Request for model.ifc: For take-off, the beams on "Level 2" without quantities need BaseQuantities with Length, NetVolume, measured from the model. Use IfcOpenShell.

First a look at what the model holds.

```python
import ifcopenshell
import ifcopenshell.util.element
import ifcopenshell.util.unit

model = ifcopenshell.open("model.ifc")
print(model.schema)
for unit_type in ("LENGTHUNIT", "AREAUNIT", "VOLUMEUNIT"):
    print(unit_type, ifcopenshell.util.unit.calculate_unit_scale(model, unit_type))
storey = next(s for s in model.by_type("IfcBuildingStorey") if s.Name == "Level 2")
beams = [e for e in ifcopenshell.util.element.get_decomposition(storey) if e.is_a("IfcBeam")]
for e in sorted(beams, key=lambda e: e.id()):
    print(e.id(), e.is_a(), e.Name, list(ifcopenshell.util.element.get_psets(e, qtos_only=True)), sep=" | ")
```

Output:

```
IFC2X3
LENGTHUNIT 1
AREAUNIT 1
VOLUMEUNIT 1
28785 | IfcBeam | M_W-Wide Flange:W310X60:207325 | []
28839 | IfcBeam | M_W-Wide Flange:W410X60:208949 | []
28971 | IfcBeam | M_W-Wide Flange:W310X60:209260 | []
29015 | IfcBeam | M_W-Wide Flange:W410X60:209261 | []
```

```python
import ifcopenshell
import ifcopenshell.api.pset
import ifcopenshell.geom
import ifcopenshell.util.element
import ifcopenshell.util.shape
import ifcopenshell.util.unit

model = ifcopenshell.open("model.ifc")
unit_scale = ifcopenshell.util.unit.calculate_unit_scale(model)
volume_scale = ifcopenshell.util.unit.calculate_unit_scale(model, "VOLUMEUNIT")
settings = ifcopenshell.geom.settings()

storey = next(s for s in model.by_type("IfcBuildingStorey") if s.Name == "Level 2")
beams = [e for e in ifcopenshell.util.element.get_decomposition(storey) if e.is_a("IfcBeam")]

for e in sorted(beams, key=lambda e: e.id()):
    if ifcopenshell.util.element.get_psets(e, qtos_only=True, should_inherit=False):
        continue
    # Geometry comes back in metres, in the element's own axes.
    shape = ifcopenshell.geom.create_shape(settings, e)
    values = {
        "Length": ifcopenshell.util.shape.get_max_xyz(shape.geometry) / unit_scale,
        "NetVolume": ifcopenshell.util.shape.get_volume(shape.geometry) / volume_scale,
    }
    qto = ifcopenshell.api.pset.add_qto(model, product=e, name="BaseQuantities")
    ifcopenshell.api.pset.edit_qto(model, qto=qto, properties=values)
    print(e.id(), {k: round(v, 3) for k, v in values.items()})

model.write("model-out.ifc")
```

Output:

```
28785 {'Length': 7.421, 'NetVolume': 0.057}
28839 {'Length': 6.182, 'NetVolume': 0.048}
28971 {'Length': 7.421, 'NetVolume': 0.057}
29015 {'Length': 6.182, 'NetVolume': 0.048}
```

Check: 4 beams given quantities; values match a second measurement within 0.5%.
